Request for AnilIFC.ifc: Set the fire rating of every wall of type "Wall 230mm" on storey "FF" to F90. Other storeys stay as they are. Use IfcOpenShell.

First a look at what the model holds.

```python
import ifcopenshell
import ifcopenshell.util.element

model = ifcopenshell.open("AnilIFC.ifc")
print(model.schema)
storey = next(s for s in model.by_type("IfcBuildingStorey") if s.Name == "FF")
walls = [e for e in ifcopenshell.util.element.get_decomposition(storey) if e.is_a("IfcWall")]
seen = {}
for e in walls:
    element_type = ifcopenshell.util.element.get_type(e)
    key = (element_type.Name if element_type != e and element_type else None, ifcopenshell.util.element.get_pset(e, "Pset_WallCommon", "FireRating"))
    seen[key] = seen.get(key, 0) + 1
for (name, value), count in sorted(seen.items(), key=str):
    print(count, "x", name, "|", value)
```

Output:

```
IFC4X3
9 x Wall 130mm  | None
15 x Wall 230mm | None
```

```python
import ifcopenshell
import ifcopenshell.api.pset
import ifcopenshell.util.element

model = ifcopenshell.open("AnilIFC.ifc")

storey = next(s for s in model.by_type("IfcBuildingStorey") if s.Name == "FF")
walls = [e for e in ifcopenshell.util.element.get_decomposition(storey) if e.is_a("IfcWall")]

count = 0
for e in walls:
    element_type = ifcopenshell.util.element.get_type(e)
    if element_type in (None, e) or element_type.Name != "Wall 230mm":
        continue
    # add_pset returns the element's existing set when there is one.
    pset = ifcopenshell.api.pset.add_pset(model, product=e, name="Pset_WallCommon")
    ifcopenshell.api.pset.edit_pset(model, pset=pset, properties={"FireRating": "F90"})
    count += 1

print(count, "walls updated")

model.write("AnilIFC_rev.ifc")
```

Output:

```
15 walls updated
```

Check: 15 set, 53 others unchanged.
